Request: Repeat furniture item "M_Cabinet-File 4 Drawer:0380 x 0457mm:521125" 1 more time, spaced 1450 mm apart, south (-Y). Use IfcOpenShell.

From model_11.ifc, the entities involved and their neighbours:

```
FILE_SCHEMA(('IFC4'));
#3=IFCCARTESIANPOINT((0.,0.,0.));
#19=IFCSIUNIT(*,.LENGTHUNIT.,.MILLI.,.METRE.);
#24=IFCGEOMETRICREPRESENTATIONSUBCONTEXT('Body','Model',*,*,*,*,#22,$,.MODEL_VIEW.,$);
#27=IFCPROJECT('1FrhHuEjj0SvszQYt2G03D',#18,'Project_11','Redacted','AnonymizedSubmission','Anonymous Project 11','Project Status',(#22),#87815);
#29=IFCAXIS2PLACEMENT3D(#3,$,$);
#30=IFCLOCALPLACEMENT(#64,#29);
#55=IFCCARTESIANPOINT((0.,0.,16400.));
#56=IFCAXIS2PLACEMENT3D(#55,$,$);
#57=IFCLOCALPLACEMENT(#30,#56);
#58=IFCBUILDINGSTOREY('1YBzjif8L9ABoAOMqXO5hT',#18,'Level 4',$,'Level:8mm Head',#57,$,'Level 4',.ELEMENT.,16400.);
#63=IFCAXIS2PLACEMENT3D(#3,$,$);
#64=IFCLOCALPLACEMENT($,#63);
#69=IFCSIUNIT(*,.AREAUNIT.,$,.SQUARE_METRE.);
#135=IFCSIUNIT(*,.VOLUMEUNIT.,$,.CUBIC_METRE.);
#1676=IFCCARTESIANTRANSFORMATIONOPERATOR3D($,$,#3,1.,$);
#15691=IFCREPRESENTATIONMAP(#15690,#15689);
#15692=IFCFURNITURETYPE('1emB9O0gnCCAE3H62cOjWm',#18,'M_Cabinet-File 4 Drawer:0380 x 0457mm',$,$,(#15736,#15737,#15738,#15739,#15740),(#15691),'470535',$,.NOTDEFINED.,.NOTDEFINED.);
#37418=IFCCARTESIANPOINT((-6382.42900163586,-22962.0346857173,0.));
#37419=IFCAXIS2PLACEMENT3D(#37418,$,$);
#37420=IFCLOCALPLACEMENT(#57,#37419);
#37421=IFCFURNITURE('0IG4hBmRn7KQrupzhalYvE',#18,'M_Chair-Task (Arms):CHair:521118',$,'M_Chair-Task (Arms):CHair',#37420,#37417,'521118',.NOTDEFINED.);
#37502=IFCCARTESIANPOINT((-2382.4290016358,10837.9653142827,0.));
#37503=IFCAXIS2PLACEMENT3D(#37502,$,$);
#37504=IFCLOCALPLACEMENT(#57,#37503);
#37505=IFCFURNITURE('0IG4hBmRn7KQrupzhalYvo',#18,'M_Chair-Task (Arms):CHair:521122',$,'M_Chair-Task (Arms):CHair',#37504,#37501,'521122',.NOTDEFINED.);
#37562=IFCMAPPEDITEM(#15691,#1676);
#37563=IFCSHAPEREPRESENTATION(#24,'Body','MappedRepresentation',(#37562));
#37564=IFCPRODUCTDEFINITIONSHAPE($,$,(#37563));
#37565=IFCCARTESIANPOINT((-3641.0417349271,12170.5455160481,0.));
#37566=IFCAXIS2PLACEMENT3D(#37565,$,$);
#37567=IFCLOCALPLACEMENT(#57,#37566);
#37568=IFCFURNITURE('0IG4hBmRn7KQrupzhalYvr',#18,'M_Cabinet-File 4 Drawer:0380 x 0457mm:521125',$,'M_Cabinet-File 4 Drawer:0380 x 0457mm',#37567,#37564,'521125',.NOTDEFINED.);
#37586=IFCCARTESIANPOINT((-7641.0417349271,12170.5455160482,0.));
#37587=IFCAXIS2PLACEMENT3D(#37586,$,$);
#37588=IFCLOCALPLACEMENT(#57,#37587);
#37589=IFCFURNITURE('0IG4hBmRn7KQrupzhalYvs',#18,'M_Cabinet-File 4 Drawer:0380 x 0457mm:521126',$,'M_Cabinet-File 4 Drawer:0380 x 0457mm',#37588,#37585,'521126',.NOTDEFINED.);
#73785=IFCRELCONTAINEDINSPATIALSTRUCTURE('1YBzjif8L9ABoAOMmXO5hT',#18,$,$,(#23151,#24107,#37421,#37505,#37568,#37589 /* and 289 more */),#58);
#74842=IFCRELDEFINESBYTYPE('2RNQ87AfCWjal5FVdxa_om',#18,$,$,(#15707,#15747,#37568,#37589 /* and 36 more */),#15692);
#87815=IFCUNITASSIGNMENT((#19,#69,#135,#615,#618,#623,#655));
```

```python
import numpy as np
import ifcopenshell
import ifcopenshell.api.geometry
import ifcopenshell.api.root
import ifcopenshell.util.element
import ifcopenshell.util.placement
import ifcopenshell.util.unit

model = ifcopenshell.open("model_11.ifc")
unit_scale = ifcopenshell.util.unit.calculate_unit_scale(model)


def reuse_history(source, copy):
    """copy_class also copies each property set's owner history, people and application; keep the originals."""
    for rel in copy.IsDefinedBy:
        if rel.is_a("IfcRelDefinesByProperties") and (history := rel.RelatingPropertyDefinition.OwnerHistory):
            rel.RelatingPropertyDefinition.OwnerHistory = source.OwnerHistory
            ifcopenshell.util.element.remove_deep2(model, history)


source = model.by_id(37568)
base = ifcopenshell.util.placement.get_local_placement(source.ObjectPlacement)
step = np.array([0.0, -1.0, 0.0]) * 1.45 / unit_scale

for i in range(1, 2):
    copy = ifcopenshell.api.root.copy_class(model, product=source)
    copy.Representation = ifcopenshell.util.element.copy_deep(
        model, source.Representation, exclude=["IfcGeometricRepresentationContext", "IfcRepresentationMap"]
    )
    copy.Name = "M_Cabinet-File 4 Drawer:0380 x 0457mm"
    copy.Tag = None
    reuse_history(source, copy)
    matrix = base.copy()
    matrix[:3, 3] += i * step
    print("added at", matrix[:3, 3].round(3) + 0.0)
    ifcopenshell.api.geometry.edit_object_placement(model, product=copy, matrix=matrix, is_si=False)

model.write("model_11_updated.ifc")
```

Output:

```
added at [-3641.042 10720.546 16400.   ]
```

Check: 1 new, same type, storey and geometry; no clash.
